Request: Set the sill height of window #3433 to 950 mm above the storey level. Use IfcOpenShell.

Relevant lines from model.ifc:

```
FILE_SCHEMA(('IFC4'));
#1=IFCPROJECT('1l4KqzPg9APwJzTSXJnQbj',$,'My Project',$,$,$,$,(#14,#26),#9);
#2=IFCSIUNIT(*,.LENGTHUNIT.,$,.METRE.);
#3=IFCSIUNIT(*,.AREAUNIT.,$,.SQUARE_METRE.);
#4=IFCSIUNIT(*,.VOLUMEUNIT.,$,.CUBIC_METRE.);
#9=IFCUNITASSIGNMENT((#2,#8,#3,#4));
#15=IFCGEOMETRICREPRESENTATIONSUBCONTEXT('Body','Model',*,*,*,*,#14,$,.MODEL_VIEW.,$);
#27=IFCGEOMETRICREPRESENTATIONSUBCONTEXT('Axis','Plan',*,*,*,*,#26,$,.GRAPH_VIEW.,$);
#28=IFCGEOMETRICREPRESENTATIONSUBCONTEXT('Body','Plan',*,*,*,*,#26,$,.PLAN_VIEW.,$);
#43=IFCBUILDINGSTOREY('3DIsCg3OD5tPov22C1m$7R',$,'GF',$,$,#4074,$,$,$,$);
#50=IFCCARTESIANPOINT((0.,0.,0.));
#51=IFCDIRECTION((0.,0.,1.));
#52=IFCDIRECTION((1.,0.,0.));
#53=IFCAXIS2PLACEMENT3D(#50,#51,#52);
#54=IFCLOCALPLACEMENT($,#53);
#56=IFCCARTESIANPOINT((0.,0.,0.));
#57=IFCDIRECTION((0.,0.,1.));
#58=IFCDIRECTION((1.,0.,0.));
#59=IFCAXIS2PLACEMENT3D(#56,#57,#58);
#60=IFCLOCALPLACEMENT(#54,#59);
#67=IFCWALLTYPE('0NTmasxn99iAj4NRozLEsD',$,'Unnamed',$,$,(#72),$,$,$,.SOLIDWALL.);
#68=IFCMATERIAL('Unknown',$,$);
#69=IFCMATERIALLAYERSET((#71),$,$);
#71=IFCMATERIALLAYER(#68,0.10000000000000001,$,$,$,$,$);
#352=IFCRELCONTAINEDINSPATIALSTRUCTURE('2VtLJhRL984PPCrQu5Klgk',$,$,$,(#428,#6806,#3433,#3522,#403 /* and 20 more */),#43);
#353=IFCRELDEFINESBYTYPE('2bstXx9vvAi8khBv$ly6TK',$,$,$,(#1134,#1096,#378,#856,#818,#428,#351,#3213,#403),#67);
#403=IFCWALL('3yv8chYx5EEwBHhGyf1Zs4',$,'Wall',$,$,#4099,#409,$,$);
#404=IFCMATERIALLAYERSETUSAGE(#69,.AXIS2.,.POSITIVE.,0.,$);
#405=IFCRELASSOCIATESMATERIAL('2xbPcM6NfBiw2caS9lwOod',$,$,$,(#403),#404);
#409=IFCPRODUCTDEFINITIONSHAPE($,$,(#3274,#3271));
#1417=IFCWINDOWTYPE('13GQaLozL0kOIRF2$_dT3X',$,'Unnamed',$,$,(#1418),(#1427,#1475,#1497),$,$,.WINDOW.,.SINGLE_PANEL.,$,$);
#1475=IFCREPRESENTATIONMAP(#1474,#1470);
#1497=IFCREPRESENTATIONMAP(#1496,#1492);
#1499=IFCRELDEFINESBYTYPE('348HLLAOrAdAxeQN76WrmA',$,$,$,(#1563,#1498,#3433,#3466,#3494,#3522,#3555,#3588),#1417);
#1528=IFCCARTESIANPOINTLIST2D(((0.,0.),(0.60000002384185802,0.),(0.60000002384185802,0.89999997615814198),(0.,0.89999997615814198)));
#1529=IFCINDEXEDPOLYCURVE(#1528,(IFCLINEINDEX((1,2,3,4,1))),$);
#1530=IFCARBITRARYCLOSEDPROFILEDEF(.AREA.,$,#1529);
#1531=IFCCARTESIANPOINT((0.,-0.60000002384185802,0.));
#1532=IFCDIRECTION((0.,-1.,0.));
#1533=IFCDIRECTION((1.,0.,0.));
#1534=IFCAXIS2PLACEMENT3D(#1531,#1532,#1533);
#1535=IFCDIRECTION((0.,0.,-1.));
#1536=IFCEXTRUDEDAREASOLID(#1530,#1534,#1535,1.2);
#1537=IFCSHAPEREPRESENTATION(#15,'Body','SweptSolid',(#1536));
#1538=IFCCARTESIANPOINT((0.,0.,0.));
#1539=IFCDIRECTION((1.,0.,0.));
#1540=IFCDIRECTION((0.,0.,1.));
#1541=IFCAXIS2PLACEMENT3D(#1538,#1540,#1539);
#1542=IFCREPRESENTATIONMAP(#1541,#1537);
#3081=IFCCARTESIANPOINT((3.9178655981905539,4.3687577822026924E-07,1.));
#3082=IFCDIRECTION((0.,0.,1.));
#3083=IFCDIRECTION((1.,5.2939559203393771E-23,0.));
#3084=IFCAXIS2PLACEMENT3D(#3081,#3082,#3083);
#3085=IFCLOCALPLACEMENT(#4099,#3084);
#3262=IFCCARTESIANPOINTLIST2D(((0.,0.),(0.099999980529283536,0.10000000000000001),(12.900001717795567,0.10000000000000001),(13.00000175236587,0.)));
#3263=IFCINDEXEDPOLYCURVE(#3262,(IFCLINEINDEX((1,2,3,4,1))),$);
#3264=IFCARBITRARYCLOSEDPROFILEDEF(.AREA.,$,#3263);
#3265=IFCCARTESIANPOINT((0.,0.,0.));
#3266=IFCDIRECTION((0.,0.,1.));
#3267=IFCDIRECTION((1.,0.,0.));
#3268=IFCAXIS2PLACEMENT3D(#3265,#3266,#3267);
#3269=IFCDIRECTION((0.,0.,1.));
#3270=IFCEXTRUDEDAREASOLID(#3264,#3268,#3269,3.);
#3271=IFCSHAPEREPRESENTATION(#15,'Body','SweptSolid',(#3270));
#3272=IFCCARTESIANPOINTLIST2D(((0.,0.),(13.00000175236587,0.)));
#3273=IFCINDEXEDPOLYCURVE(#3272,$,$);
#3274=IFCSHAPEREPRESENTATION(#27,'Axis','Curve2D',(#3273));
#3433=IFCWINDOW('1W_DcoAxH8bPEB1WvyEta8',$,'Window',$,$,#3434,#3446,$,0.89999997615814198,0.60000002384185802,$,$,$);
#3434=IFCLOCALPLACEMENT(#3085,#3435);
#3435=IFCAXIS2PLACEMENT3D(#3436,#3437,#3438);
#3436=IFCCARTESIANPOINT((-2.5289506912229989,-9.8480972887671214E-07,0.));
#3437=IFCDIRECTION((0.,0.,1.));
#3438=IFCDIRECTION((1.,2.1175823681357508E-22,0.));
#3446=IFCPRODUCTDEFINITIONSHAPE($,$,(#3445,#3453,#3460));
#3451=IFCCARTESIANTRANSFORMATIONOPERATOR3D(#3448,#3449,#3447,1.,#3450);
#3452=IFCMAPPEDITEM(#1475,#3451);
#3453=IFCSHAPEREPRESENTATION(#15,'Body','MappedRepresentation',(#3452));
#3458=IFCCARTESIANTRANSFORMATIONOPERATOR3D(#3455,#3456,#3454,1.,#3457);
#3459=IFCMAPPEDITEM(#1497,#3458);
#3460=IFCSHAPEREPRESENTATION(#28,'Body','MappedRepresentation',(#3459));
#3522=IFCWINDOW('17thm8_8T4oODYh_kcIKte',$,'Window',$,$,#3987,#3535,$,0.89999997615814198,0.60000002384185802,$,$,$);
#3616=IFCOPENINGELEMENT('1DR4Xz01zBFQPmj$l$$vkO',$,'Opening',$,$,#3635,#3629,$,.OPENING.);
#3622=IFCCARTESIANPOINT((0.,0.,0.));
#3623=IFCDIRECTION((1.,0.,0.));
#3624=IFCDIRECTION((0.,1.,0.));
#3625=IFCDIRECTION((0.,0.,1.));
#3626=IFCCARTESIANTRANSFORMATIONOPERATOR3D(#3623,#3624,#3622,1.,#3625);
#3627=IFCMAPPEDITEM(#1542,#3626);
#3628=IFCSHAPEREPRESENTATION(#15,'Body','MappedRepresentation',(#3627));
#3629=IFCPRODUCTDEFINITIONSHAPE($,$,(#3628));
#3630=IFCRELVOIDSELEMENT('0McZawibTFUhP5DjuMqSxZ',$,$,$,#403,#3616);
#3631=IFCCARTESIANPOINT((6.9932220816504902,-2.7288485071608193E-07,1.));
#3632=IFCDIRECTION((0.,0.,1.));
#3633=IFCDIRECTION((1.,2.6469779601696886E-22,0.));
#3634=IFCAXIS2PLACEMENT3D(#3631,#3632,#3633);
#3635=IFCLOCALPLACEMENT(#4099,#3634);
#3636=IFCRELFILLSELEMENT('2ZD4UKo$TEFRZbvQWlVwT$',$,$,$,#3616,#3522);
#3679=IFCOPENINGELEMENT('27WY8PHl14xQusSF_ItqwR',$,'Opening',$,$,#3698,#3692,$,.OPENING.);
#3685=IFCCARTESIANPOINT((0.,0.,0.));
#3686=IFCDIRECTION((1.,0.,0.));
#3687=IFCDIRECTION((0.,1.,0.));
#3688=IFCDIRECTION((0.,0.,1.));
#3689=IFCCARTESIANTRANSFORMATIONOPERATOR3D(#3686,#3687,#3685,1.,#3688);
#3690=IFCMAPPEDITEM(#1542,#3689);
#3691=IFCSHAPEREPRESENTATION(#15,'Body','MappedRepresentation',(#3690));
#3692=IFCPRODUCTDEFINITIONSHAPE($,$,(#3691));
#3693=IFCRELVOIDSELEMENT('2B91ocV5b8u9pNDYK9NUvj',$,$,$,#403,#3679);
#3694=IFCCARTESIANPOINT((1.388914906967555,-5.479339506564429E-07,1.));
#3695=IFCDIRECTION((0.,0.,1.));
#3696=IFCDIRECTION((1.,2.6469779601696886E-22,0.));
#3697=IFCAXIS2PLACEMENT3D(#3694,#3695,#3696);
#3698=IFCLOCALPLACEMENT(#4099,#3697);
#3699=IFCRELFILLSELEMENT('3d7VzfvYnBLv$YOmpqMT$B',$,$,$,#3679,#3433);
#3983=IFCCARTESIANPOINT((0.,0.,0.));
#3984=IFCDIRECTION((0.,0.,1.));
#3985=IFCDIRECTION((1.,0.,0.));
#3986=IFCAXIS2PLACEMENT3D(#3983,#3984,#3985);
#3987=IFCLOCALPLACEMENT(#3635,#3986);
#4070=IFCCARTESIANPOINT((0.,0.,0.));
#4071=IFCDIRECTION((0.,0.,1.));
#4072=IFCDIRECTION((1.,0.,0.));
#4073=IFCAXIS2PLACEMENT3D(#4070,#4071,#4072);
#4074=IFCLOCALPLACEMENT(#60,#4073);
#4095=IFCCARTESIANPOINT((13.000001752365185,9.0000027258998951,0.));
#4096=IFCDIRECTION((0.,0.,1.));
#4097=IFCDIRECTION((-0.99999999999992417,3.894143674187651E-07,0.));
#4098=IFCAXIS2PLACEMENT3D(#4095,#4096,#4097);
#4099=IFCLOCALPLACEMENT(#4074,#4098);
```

```python
import numpy as np
import ifcopenshell
import ifcopenshell.api.geometry
import ifcopenshell.geom
import ifcopenshell.util.element
import ifcopenshell.util.placement
import ifcopenshell.util.shape
import ifcopenshell.util.unit

model = ifcopenshell.open("model.ifc")
unit_scale = ifcopenshell.util.unit.calculate_unit_scale(model)

window = model.by_guid("1W_DcoAxH8bPEB1WvyEta8")
opening = window.FillsVoids[0].RelatingOpeningElement
storey = ifcopenshell.util.element.get_container(window, ifc_class="IfcBuildingStorey")
level = ifcopenshell.util.placement.get_local_placement(storey.ObjectPlacement)[2, 3]

# The opening's origin need not be at the sill, so measure its lowest point.
shape = ifcopenshell.geom.create_shape(ifcopenshell.geom.settings(), opening)
bottom = ifcopenshell.util.shape.get_shape_bottom_elevation(shape, shape.geometry) / unit_scale
dz = level + 0.95 / unit_scale - bottom

shift = np.array([0.0, 0.0, dz])
# The window is not placed relative to its opening, so move both.
for product in (opening, window):
    matrix = ifcopenshell.util.placement.get_local_placement(product.ObjectPlacement)
    matrix[:3, 3] += shift
    ifcopenshell.api.geometry.edit_object_placement(model, product=product, matrix=matrix, is_si=False)

print(f"moved by {dz * unit_scale:+.3f} m")

model.write("model_updated.ifc")
```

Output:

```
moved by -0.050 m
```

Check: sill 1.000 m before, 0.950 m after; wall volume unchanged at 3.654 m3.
